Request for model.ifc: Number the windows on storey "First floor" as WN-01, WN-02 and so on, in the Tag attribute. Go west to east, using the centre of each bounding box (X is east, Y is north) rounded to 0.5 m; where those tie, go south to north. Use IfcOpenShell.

First a look at what the model holds.

```python
import ifcopenshell
import ifcopenshell.util.element
import ifcopenshell.util.placement

model = ifcopenshell.open("model.ifc")
print(model.schema)
storey = next(s for s in model.by_type("IfcBuildingStorey") if s.Name == "First floor")
windows = [e for e in ifcopenshell.util.element.get_decomposition(storey) if e.is_a("IfcWindow")]
for e in sorted(windows, key=lambda e: e.id()):
    origin = ifcopenshell.util.placement.get_local_placement(e.ObjectPlacement)[:3, 3]
    print(e.id(), e.Tag, e.Name, origin.round(2) + 0.0, sep=" | ")
```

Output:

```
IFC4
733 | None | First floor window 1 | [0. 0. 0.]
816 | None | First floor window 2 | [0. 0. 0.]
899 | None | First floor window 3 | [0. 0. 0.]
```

```python
import ifcopenshell
import ifcopenshell.geom
import ifcopenshell.util.element
import ifcopenshell.util.shape

model = ifcopenshell.open("model.ifc")
settings = ifcopenshell.geom.settings()
settings.set("use-world-coords", True)


def centre(element):
    shape = ifcopenshell.geom.create_shape(settings, element)
    return ifcopenshell.util.shape.get_bbox_centroid(shape.geometry)


storey = next(s for s in model.by_type("IfcBuildingStorey") if s.Name == "First floor")
windows = [e for e in ifcopenshell.util.element.get_decomposition(storey) if e.is_a("IfcWindow")]

# Insertion points can sit at a corner or the storey origin, so sort by the geometry (in metres).
centres = {e: centre(e) for e in windows}
windows.sort(key=lambda e: (round(centres[e][0] / 0.5), centres[e][1]))

for i, e in enumerate(windows, start=1):
    number = f"WN-{i:02d}"
    e.Tag = number
    print(e.id(), number)

model.write("model_rev.ifc")
```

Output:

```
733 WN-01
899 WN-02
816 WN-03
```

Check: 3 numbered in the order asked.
